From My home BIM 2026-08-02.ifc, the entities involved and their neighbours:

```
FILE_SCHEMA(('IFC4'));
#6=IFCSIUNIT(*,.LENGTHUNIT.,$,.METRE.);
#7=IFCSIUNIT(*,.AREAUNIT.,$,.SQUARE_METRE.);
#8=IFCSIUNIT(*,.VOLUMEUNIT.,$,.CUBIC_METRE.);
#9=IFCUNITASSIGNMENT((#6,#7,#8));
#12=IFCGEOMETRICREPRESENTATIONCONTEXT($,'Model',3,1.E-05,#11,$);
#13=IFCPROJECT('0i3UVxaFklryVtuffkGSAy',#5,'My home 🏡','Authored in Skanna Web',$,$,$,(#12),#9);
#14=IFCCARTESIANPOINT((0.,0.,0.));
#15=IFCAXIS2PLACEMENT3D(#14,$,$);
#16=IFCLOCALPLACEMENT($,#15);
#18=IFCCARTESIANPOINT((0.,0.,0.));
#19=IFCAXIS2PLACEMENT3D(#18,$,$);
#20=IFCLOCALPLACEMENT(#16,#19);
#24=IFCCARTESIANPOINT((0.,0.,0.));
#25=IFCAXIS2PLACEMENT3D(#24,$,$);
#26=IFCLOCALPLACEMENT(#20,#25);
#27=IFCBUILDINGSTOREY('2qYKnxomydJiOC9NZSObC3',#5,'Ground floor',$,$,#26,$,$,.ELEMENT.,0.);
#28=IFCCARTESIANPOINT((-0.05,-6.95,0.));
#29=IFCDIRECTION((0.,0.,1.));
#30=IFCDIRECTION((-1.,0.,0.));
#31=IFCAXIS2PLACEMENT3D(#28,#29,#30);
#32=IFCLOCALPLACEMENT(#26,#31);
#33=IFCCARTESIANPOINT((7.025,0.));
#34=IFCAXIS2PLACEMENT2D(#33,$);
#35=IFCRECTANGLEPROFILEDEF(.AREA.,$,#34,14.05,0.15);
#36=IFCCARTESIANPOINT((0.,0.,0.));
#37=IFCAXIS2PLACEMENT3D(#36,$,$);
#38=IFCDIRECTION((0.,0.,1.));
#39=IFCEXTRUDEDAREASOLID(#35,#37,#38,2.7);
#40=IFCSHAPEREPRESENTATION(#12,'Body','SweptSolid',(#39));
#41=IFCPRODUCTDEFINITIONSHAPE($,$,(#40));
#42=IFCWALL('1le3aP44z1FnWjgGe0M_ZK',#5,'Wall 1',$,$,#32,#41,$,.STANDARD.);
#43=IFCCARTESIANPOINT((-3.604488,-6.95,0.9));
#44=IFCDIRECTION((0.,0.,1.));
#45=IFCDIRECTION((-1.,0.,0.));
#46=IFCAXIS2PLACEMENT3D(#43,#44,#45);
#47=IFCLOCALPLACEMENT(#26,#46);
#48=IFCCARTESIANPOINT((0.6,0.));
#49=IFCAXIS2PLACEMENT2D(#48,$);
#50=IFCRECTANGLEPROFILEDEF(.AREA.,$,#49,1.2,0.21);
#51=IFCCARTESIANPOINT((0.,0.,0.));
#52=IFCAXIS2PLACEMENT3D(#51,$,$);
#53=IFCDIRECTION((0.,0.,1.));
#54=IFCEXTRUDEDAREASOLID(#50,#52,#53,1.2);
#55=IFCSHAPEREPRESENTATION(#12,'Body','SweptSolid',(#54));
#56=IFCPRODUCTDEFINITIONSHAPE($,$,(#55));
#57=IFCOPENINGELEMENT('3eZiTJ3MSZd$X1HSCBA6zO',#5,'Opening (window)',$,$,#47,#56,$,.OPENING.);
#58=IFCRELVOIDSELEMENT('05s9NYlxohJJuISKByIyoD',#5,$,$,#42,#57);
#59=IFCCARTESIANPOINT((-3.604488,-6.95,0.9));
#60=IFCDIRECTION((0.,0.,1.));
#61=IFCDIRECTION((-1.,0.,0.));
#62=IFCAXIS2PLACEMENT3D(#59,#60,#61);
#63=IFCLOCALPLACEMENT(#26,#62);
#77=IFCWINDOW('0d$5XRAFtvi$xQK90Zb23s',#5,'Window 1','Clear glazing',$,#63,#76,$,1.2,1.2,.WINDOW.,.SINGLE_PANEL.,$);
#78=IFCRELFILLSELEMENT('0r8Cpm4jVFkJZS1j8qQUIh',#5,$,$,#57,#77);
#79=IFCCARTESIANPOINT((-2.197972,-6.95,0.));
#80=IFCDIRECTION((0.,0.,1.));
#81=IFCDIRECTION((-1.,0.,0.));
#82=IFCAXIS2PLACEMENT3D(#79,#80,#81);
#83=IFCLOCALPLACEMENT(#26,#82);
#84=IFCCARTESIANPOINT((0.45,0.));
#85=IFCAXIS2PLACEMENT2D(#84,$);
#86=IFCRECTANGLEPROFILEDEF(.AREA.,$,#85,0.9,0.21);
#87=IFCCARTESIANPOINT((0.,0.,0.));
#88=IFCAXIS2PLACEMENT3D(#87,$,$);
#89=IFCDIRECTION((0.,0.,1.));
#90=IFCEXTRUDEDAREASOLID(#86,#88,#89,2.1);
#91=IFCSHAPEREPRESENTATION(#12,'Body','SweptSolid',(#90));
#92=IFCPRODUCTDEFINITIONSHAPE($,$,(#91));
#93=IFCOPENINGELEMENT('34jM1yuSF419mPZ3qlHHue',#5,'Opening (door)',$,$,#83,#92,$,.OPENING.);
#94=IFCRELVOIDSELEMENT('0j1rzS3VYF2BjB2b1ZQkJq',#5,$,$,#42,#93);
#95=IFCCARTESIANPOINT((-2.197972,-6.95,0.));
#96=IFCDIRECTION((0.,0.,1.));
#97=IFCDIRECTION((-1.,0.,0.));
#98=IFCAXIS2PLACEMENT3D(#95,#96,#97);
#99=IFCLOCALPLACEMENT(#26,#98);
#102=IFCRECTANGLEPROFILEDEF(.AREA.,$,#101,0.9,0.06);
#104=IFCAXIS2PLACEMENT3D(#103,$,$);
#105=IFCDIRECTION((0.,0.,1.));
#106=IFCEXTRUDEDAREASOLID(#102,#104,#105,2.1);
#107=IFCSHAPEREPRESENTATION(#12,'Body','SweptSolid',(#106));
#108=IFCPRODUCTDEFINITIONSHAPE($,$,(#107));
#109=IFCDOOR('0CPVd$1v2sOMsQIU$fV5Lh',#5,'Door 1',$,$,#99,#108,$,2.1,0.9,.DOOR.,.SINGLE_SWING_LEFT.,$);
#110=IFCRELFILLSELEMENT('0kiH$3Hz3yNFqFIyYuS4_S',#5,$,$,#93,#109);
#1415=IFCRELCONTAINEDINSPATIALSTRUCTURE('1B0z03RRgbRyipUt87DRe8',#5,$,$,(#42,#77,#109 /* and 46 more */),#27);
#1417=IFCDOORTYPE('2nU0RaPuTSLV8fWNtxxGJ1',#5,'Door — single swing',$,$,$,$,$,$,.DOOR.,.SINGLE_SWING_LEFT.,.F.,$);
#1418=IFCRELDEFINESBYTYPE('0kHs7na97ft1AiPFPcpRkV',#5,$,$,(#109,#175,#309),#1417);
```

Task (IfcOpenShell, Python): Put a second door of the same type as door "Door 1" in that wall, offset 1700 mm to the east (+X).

```python
import ifcopenshell
import ifcopenshell.api.feature
import ifcopenshell.api.geometry
import ifcopenshell.api.root
import ifcopenshell.geom
import ifcopenshell.util.element
import ifcopenshell.util.placement
import ifcopenshell.util.shape
import ifcopenshell.util.unit

model = ifcopenshell.open("My home BIM 2026-08-02.ifc")
unit_scale = ifcopenshell.util.unit.calculate_unit_scale(model)
settings = ifcopenshell.geom.settings()


def volume(element):
    """Net volume in cubic metres, openings subtracted."""
    shape = ifcopenshell.geom.create_shape(settings, element)
    return ifcopenshell.util.shape.get_volume(shape.geometry)


door = model.by_guid("0CPVd$1v2sOMsQIU$fV5Lh")
opening = door.FillsVoids[0].RelatingOpeningElement
wall = opening.VoidsElements[0].RelatingBuildingElement
before = volume(wall)
shift = ifcopenshell.util.placement.get_local_placement(wall.ObjectPlacement)[:3, 0] * -1.7 / unit_scale

# copy_class copies the void relationship, type, container and properties, but no geometry.
new_opening = ifcopenshell.api.root.copy_class(model, product=opening)
new_opening.Representation = ifcopenshell.util.element.copy_deep(
    model, opening.Representation, exclude=["IfcGeometricRepresentationContext", "IfcRepresentationMap"]
)
new_door = ifcopenshell.api.root.copy_class(model, product=door)
new_door.Representation = ifcopenshell.util.element.copy_deep(
    model, door.Representation, exclude=["IfcGeometricRepresentationContext", "IfcRepresentationMap"]
)
ifcopenshell.api.feature.add_filling(model, opening=new_opening, element=new_door)

for old, new in ((opening, new_opening), (door, new_door)):
    matrix = ifcopenshell.util.placement.get_local_placement(old.ObjectPlacement)
    matrix[:3, 3] += shift
    ifcopenshell.api.geometry.edit_object_placement(model, product=new, matrix=matrix, is_si=False)

after = volume(wall)

print(f"wall volume {before:.3f} -> {after:.3f} m3")

model.write("My home BIM 2026-08-02_rev.ifc")
```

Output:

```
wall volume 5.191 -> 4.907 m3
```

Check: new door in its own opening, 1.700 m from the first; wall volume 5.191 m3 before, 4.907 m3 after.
